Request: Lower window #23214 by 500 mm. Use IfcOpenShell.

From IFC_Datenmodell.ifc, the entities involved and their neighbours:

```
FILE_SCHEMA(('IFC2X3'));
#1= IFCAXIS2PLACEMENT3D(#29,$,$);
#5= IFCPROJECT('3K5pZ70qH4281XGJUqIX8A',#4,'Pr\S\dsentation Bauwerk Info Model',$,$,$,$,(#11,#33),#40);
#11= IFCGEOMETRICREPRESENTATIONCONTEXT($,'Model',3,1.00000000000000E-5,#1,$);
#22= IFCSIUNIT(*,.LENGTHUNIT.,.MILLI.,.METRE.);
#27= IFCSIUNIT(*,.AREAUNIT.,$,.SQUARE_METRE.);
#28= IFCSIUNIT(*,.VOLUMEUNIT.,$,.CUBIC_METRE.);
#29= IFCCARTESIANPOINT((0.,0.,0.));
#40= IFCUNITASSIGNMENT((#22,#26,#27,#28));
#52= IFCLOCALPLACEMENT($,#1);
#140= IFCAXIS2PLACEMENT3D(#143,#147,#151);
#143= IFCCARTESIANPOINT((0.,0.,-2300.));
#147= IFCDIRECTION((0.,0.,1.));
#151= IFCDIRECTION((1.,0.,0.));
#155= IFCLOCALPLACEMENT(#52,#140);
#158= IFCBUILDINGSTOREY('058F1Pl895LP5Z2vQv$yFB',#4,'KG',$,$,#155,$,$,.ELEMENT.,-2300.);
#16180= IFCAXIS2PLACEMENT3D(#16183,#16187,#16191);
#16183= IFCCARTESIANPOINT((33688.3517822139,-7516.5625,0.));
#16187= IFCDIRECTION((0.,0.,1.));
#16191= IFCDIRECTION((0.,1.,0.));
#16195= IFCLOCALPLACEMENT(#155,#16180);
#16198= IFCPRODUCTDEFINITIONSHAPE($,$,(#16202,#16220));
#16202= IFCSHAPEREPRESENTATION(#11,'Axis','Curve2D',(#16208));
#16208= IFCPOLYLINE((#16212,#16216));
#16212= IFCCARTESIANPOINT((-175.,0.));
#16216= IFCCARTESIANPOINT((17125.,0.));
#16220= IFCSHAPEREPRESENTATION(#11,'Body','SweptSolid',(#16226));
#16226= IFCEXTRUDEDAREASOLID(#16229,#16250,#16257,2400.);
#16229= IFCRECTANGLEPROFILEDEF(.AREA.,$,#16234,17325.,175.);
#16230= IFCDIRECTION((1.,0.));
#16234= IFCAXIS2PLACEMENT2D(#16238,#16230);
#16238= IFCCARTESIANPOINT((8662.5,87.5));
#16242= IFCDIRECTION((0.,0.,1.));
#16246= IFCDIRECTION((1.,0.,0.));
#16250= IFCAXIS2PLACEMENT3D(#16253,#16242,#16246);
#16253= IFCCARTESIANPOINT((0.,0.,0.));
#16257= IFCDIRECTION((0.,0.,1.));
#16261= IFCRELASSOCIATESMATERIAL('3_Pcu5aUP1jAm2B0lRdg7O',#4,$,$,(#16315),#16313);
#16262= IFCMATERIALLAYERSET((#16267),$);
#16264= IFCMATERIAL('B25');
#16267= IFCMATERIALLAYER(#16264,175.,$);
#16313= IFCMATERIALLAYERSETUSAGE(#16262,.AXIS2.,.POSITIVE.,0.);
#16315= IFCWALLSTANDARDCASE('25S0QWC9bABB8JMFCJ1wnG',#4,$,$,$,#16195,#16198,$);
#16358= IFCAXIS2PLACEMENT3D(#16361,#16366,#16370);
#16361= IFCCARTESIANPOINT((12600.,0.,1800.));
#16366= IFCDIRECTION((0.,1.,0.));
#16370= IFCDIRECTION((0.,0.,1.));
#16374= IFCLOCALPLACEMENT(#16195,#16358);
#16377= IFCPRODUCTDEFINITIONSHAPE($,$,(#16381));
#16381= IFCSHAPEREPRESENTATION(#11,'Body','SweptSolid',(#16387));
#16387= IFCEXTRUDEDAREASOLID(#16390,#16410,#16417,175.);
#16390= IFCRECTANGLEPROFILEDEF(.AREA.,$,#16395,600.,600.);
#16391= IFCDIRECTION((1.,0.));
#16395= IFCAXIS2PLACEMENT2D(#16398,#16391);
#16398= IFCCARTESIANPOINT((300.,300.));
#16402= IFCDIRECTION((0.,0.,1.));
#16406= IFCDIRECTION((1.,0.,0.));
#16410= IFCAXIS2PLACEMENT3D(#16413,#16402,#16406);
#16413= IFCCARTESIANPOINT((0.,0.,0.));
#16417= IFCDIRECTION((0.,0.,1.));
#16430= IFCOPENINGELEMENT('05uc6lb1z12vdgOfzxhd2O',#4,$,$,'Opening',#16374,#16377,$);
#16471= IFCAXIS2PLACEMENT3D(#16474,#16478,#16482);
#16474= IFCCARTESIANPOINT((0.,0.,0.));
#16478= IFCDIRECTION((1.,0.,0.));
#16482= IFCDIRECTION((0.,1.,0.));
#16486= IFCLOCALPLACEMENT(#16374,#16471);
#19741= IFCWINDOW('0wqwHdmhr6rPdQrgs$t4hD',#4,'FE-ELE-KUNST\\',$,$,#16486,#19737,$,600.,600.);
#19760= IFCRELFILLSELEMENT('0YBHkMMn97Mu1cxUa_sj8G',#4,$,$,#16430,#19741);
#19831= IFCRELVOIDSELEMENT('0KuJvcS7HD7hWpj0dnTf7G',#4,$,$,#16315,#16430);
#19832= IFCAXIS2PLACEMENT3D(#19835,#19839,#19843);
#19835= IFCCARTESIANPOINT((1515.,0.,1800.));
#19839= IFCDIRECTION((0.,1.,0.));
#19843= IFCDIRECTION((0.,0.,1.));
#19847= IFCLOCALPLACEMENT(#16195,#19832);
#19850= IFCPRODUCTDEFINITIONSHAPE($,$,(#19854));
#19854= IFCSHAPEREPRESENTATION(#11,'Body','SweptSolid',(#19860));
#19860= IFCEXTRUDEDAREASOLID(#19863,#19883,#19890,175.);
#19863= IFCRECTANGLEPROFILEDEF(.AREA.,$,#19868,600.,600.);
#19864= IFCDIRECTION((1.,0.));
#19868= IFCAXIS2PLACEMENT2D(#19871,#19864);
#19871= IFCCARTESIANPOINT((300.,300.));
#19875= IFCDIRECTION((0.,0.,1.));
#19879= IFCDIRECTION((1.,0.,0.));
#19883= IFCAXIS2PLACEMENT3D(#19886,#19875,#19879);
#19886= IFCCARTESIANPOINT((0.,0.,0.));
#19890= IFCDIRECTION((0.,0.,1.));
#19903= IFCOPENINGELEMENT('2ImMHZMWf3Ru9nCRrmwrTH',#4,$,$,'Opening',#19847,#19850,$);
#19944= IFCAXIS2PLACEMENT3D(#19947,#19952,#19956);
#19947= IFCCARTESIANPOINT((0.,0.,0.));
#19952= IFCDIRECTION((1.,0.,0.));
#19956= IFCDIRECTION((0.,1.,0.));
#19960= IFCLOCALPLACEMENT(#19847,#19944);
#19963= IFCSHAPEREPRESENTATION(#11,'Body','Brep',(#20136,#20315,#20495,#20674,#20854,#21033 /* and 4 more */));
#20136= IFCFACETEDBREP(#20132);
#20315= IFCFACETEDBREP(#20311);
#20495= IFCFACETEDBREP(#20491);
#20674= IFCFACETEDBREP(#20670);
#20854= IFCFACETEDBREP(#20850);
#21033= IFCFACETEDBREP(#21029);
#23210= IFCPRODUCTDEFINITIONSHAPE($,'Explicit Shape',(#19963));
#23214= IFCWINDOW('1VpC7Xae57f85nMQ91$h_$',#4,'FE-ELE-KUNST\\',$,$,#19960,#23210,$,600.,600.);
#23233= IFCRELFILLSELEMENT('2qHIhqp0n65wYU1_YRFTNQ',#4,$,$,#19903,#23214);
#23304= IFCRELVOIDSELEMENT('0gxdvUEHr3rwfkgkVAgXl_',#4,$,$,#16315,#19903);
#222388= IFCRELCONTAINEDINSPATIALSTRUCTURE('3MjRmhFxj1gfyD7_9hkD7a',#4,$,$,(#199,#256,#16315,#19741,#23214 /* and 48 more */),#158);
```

```python
import numpy as np
import ifcopenshell
import ifcopenshell.api.geometry
import ifcopenshell.util.placement
import ifcopenshell.util.unit

model = ifcopenshell.open("IFC_Datenmodell.ifc")
unit_scale = ifcopenshell.util.unit.calculate_unit_scale(model)

window = model.by_guid("1VpC7Xae57f85nMQ91$h_$")
opening = window.FillsVoids[0].RelatingOpeningElement
dz = -500.0

shift = np.array([0.0, 0.0, dz])
# The window is placed relative to its opening, so it follows when the opening moves.
matrix = ifcopenshell.util.placement.get_local_placement(opening.ObjectPlacement)
matrix[:3, 3] += shift
ifcopenshell.api.geometry.edit_object_placement(
    model, product=opening, matrix=matrix, is_si=False, should_transform_children=True
)

print(f"moved by {dz * unit_scale:+.3f} m")

model.write("IFC_Datenmodell_rev.ifc")
```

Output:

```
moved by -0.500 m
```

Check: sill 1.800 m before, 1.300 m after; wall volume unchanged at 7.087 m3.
